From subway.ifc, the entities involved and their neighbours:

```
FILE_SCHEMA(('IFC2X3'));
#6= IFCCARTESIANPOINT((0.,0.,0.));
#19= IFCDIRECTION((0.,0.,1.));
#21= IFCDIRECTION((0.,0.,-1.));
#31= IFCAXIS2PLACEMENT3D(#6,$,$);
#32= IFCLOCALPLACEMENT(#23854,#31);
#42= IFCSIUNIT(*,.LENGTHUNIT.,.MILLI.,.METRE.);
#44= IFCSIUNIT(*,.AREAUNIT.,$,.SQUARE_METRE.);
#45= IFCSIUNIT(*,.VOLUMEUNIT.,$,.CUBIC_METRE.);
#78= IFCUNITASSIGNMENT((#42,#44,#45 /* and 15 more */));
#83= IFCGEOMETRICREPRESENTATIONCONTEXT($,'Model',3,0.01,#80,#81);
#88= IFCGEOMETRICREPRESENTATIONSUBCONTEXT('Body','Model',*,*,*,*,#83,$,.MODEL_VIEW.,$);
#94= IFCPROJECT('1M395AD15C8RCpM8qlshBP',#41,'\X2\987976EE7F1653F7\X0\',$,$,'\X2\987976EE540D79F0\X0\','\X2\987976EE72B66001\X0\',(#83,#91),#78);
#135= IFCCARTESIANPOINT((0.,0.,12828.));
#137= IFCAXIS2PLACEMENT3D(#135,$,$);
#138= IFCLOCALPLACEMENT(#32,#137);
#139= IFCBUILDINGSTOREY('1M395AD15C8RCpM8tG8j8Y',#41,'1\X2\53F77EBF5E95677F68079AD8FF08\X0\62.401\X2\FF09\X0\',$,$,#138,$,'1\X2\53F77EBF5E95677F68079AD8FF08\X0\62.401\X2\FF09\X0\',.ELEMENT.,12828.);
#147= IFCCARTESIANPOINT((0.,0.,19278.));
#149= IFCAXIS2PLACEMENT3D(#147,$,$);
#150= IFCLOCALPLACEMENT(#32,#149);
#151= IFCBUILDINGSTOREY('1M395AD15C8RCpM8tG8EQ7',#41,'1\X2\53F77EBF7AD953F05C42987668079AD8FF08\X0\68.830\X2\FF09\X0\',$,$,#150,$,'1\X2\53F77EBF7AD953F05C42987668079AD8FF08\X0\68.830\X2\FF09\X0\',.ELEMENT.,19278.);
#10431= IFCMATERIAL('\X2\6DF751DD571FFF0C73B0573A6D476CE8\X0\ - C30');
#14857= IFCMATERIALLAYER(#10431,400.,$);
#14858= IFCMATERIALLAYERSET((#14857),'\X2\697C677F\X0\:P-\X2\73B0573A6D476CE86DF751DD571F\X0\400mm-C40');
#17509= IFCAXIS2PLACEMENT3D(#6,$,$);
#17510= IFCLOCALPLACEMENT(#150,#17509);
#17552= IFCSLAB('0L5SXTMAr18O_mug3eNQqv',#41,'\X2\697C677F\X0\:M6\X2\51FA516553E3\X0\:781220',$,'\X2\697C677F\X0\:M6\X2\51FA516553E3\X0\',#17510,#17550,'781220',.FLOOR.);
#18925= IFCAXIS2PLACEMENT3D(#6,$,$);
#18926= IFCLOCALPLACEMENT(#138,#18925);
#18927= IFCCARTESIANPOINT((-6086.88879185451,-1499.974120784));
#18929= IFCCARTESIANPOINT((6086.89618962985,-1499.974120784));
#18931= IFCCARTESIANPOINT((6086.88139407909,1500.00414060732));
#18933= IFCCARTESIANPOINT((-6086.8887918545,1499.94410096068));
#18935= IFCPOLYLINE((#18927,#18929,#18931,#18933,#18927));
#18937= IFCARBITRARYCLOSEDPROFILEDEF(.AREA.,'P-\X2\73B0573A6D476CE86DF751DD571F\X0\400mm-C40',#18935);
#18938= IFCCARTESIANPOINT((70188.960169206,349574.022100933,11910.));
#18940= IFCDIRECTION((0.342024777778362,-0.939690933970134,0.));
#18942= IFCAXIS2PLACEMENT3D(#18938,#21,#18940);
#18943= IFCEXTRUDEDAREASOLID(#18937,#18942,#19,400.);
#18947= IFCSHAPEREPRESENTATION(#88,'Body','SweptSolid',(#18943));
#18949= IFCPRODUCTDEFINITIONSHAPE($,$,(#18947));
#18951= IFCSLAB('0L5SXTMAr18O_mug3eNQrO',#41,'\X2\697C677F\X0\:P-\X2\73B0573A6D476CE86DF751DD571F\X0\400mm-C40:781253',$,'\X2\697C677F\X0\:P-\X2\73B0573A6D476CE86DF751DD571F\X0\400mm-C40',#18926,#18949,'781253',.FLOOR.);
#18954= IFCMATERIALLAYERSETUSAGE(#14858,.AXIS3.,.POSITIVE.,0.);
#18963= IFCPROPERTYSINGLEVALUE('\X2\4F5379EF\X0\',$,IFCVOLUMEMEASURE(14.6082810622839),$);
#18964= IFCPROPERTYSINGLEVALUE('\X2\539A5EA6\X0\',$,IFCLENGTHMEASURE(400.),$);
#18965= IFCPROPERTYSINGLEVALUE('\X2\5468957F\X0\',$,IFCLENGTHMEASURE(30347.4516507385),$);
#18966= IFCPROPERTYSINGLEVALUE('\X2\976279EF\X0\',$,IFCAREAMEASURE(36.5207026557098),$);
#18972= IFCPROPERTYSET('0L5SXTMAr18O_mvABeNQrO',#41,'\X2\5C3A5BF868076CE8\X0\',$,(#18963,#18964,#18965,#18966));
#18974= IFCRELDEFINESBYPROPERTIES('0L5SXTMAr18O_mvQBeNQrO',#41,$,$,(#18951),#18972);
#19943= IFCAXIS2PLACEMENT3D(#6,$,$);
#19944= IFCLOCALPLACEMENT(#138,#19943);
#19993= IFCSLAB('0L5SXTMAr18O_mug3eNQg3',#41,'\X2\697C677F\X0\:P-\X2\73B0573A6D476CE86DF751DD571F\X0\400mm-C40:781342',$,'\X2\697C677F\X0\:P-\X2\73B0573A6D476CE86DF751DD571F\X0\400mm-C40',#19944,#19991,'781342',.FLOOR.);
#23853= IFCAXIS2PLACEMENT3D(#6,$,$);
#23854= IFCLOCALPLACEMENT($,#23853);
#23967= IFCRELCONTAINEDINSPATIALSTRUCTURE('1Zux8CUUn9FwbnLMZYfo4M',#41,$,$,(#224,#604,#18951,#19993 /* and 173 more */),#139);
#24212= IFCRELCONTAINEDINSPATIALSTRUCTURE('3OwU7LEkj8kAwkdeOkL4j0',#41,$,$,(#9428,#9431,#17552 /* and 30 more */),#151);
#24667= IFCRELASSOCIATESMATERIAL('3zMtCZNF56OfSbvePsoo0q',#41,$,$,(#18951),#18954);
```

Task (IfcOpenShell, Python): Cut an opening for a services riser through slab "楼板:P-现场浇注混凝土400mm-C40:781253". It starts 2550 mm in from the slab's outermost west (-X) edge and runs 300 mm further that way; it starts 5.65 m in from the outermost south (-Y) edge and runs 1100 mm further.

```python
import numpy as np
import ifcopenshell
import ifcopenshell.api.feature
import ifcopenshell.api.geometry
import ifcopenshell.api.pset
import ifcopenshell.api.root
import ifcopenshell.geom
import ifcopenshell.util.element
import ifcopenshell.util.placement
import ifcopenshell.util.representation
import ifcopenshell.util.shape
import ifcopenshell.util.unit

model = ifcopenshell.open("subway.ifc")
unit_scale = ifcopenshell.util.unit.calculate_unit_scale(model)
area_scale = ifcopenshell.util.unit.calculate_unit_scale(model, "AREAUNIT")
volume_scale = ifcopenshell.util.unit.calculate_unit_scale(model, "VOLUMEUNIT")
settings = ifcopenshell.geom.settings()


def volume(element):
    """Net volume in cubic metres, openings subtracted."""
    shape = ifcopenshell.geom.create_shape(settings, element)
    return ifcopenshell.util.shape.get_volume(shape.geometry)


slab = model.by_guid("0L5SXTMAr18O_mug3eNQrO")
before = volume(slab)

# Extent in the slab's own axes, in metres. The edges named are its -X and -Y sides.
slab_shape = ifcopenshell.geom.create_shape(settings, slab)
vertices = ifcopenshell.util.shape.get_vertices(slab_shape.geometry)
x_min, y_min, bottom = vertices.min(axis=0)
top = vertices[:, 2].max()

opening = ifcopenshell.api.root.create_entity(model, ifc_class="IfcOpeningElement", name="Services riser opening")
context = ifcopenshell.util.representation.get_context(model, "Model", "Body", "MODEL_VIEW")
width, depth = 0.3, 1.1
outline = [(0.0, 0.0), (width, 0.0), (width, depth), (0.0, depth), (0.0, 0.0)]
# Overshoot both faces by 50 mm so the cut is clean.
shape = ifcopenshell.api.geometry.add_slab_representation(
    model, context=context, depth=top - bottom + 0.1, polyline=outline
)
ifcopenshell.api.geometry.assign_representation(model, product=opening, representation=shape)

matrix = ifcopenshell.util.placement.get_local_placement(slab.ObjectPlacement)
matrix[:, 3] = matrix @ np.append(np.array([x_min + 2.55, y_min + 5.65, bottom - 0.05]) / unit_scale, 1.0)
ifcopenshell.api.geometry.edit_object_placement(model, product=opening, matrix=matrix, is_si=False)
ifcopenshell.api.feature.add_feature(model, feature=opening, element=slab)

after = volume(slab)

# Update the slab's stored quantities.
pset = model.by_id(ifcopenshell.util.element.get_pset(slab, "尺寸标注", should_inherit=False)["id"])
ifcopenshell.api.pset.edit_pset(model, pset=pset, properties={
    "体积": model.create_entity("IfcVolumeMeasure", after / volume_scale),
    "面积": model.create_entity("IfcAreaMeasure", after / (top - bottom) / area_scale),
})

print(f"slab volume {before:.3f} -> {after:.3f} m3")

model.write("subway-out.ifc")
```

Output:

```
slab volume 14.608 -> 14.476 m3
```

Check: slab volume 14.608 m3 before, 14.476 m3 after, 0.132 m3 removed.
